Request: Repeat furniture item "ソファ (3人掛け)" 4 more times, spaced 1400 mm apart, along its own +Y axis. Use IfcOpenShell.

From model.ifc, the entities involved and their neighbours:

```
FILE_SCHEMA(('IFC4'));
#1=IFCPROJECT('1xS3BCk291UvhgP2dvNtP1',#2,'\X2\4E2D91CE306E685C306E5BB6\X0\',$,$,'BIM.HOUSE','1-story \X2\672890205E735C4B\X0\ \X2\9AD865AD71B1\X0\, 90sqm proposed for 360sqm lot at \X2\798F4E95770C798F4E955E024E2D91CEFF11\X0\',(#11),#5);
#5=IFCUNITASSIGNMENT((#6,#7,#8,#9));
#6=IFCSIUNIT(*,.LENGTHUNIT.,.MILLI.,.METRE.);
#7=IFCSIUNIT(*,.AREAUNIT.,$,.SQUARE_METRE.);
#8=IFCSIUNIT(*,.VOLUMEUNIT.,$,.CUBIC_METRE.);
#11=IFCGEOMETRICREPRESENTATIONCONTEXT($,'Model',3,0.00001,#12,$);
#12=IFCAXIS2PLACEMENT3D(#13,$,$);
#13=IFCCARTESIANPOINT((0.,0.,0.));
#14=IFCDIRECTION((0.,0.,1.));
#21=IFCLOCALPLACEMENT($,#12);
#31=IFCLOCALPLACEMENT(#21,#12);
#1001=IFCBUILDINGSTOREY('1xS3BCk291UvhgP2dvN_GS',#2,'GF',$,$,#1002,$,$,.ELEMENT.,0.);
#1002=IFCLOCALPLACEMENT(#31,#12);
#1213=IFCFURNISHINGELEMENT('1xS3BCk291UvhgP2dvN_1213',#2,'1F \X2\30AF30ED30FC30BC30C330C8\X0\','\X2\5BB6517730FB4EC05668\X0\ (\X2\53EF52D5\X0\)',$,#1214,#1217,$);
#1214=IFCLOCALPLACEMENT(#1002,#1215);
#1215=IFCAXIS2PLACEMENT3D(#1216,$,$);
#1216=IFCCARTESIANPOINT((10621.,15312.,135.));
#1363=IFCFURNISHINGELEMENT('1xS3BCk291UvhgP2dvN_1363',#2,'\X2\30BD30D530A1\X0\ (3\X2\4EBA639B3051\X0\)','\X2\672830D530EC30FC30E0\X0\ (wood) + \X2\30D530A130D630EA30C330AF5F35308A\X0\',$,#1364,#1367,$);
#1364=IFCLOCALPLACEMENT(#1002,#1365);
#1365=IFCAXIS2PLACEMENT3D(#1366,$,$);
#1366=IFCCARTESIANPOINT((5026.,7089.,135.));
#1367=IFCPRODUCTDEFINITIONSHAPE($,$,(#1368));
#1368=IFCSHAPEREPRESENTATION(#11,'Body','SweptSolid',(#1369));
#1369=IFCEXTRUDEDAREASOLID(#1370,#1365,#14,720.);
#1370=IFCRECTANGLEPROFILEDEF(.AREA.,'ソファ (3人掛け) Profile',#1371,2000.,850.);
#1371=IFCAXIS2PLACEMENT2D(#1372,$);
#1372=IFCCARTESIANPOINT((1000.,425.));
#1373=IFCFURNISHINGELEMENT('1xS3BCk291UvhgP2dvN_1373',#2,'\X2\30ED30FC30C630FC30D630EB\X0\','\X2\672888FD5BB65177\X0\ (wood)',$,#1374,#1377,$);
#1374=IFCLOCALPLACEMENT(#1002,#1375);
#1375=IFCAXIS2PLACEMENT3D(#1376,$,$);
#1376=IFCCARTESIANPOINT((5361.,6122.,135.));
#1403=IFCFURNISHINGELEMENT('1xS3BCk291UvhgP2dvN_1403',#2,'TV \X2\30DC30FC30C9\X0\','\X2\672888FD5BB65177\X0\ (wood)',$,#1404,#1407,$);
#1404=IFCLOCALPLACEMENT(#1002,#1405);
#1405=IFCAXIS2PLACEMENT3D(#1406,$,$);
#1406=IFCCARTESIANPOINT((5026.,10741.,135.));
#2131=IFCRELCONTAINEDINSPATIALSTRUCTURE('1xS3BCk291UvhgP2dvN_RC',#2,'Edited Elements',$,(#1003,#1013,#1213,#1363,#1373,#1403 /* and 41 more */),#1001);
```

```python
import ifcopenshell
import ifcopenshell.api.geometry
import ifcopenshell.api.root
import ifcopenshell.util.element
import ifcopenshell.util.placement

model = ifcopenshell.open("model.ifc")


def reuse_history(source, copy):
    """copy_class also copies each property set's owner history, people and application; keep the originals."""
    for rel in copy.IsDefinedBy:
        if rel.is_a("IfcRelDefinesByProperties") and (history := rel.RelatingPropertyDefinition.OwnerHistory):
            rel.RelatingPropertyDefinition.OwnerHistory = source.OwnerHistory
            ifcopenshell.util.element.remove_deep2(model, history)


source = model.by_guid("1xS3BCk291UvhgP2dvN_1363")
base = ifcopenshell.util.placement.get_local_placement(source.ObjectPlacement)
step = base[:3, 1] * 1400.0

for i in range(1, 5):
    copy = ifcopenshell.api.root.copy_class(model, product=source)
    copy.Representation = ifcopenshell.util.element.copy_deep(
        model, source.Representation, exclude=["IfcGeometricRepresentationContext", "IfcRepresentationMap"]
    )
    reuse_history(source, copy)
    matrix = base.copy()
    matrix[:3, 3] += i * step
    print("added at", matrix[:3, 3].round(3) + 0.0)
    ifcopenshell.api.geometry.edit_object_placement(model, product=copy, matrix=matrix, is_si=False)

model.write("model_updated.ifc")
```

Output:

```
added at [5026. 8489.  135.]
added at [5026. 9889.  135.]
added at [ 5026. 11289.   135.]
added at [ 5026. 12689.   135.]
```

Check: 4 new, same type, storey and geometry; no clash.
